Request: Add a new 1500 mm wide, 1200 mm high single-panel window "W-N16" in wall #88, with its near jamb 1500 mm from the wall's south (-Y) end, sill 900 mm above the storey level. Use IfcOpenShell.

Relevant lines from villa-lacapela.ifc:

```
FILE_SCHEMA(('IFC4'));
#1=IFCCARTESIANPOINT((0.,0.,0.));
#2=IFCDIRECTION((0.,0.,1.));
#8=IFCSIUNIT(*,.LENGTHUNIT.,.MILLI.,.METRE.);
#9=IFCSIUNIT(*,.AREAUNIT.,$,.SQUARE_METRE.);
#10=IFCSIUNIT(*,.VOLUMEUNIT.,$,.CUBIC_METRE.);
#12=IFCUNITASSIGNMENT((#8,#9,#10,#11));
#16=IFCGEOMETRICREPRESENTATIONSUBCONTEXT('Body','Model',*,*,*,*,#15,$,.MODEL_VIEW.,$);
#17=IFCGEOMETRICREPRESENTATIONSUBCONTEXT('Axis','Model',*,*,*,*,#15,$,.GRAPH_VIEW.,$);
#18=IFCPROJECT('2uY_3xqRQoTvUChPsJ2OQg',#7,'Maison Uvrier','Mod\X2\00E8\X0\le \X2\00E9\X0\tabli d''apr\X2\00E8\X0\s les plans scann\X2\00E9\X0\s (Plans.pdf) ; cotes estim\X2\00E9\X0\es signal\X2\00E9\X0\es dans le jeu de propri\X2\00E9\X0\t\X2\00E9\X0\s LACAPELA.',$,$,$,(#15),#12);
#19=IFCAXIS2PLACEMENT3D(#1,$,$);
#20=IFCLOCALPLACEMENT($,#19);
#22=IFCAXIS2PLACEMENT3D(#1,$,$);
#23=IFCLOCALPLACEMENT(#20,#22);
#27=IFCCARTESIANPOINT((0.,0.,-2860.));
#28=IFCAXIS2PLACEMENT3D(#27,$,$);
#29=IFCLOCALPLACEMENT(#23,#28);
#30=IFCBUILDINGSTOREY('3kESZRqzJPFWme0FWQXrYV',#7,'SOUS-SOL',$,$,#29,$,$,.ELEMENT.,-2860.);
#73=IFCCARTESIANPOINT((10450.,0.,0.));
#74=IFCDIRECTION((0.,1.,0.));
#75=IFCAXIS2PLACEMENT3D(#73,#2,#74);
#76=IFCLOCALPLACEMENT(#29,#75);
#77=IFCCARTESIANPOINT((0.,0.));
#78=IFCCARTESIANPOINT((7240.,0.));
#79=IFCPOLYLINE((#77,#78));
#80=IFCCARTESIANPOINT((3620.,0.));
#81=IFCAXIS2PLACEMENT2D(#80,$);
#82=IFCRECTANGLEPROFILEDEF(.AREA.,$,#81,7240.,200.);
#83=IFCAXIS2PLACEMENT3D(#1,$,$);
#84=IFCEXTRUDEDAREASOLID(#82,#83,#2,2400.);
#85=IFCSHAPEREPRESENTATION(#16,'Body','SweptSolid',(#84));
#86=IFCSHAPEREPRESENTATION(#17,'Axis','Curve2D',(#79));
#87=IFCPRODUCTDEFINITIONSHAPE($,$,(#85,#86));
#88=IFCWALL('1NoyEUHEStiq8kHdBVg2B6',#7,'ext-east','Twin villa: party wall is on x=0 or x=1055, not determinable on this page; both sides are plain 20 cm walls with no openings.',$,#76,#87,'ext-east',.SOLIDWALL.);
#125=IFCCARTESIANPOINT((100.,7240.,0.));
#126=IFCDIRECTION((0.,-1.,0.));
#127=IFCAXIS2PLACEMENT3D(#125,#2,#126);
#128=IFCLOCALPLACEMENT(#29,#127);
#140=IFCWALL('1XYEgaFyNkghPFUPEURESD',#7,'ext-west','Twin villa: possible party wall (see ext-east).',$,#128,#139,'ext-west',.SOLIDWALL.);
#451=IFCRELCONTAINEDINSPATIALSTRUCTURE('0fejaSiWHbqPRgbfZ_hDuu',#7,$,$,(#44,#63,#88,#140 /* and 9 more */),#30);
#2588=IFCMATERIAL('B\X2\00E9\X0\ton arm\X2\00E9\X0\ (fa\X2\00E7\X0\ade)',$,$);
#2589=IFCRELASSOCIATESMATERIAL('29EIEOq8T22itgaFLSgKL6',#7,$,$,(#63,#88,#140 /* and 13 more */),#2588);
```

```python
import numpy as np
import ifcopenshell
import ifcopenshell.api.feature
import ifcopenshell.api.geometry
import ifcopenshell.api.root
import ifcopenshell.api.spatial
import ifcopenshell.geom
import ifcopenshell.util.element
import ifcopenshell.util.placement
import ifcopenshell.util.representation
import ifcopenshell.util.shape
import ifcopenshell.util.unit

model = ifcopenshell.open("villa-lacapela.ifc")
unit_scale = ifcopenshell.util.unit.calculate_unit_scale(model)
settings = ifcopenshell.geom.settings()


def volume(element):
    """Net volume in cubic metres, openings subtracted."""
    shape = ifcopenshell.geom.create_shape(settings, element)
    return ifcopenshell.util.shape.get_volume(shape.geometry)


wall = model.by_guid("1NoyEUHEStiq8kHdBVg2B6")
storey = ifcopenshell.util.element.get_container(wall, ifc_class="IfcBuildingStorey")
context = ifcopenshell.util.representation.get_context(model, "Model", "Body", "MODEL_VIEW")
before = volume(wall)

width, height, from_end, sill = 1.5, 1.2, 1.5, 0.9  # metres

# The wall runs along its own X axis, and the end named is its -X end.
wall_shape = ifcopenshell.geom.create_shape(settings, wall)
x, y, z = ifcopenshell.util.shape.get_vertices(wall_shape.geometry).T
start = x.min() + from_end
face, thickness = float(y.min()), float(y.max() - y.min())
wall_matrix = ifcopenshell.util.placement.get_local_placement(wall.ObjectPlacement)
level = ifcopenshell.util.placement.get_local_placement(storey.ObjectPlacement)[2, 3]


def in_wall(x, y):
    """Placement at x, y metres in the wall's axes, at sill height."""
    matrix = wall_matrix.copy()
    matrix[:, 3] = wall_matrix @ np.array([x / unit_scale, y / unit_scale, 0.0, 1.0])
    matrix[2, 3] = level + sill / unit_scale
    return matrix


# Opening: a box that overshoots both wall faces by 50 mm.
opening = ifcopenshell.api.root.create_entity(model, ifc_class="IfcOpeningElement", predefined_type="OPENING")
box = ifcopenshell.api.geometry.add_wall_representation(
    model, context=context, length=width, height=height, thickness=thickness + 0.1
)
ifcopenshell.api.geometry.assign_representation(model, product=opening, representation=box)
ifcopenshell.api.geometry.edit_object_placement(model, product=opening, matrix=in_wall(start, face - 0.05), is_si=False)
ifcopenshell.api.feature.add_feature(model, feature=opening, element=wall)

window = ifcopenshell.api.root.create_entity(model, ifc_class="IfcWindow", name="W-N16", predefined_type="WINDOW")
window.OverallWidth, window.OverallHeight = width / unit_scale, height / unit_scale
window.PartitioningType = "SINGLE_PANEL"
body = ifcopenshell.api.geometry.add_window_representation(
    model,
    context=context,
    overall_width=window.OverallWidth,
    overall_height=window.OverallHeight,
    partition_type="SINGLE_PANEL",
)
ifcopenshell.api.geometry.assign_representation(model, product=window, representation=body)
ifcopenshell.api.spatial.assign_container(model, products=[window], relating_structure=storey)
ifcopenshell.api.feature.add_filling(model, opening=opening, element=window)

# Centre the window in the wall's thickness.
ifcopenshell.api.geometry.edit_object_placement(model, product=window, matrix=in_wall(start, face), is_si=False)
window_shape = ifcopenshell.geom.create_shape(settings, window)
depth = ifcopenshell.util.shape.get_vertices(window_shape.geometry)[:, 1]
offset = face + thickness / 2 - (depth.min() + depth.max()) / 2
ifcopenshell.api.geometry.edit_object_placement(model, product=window, matrix=in_wall(start, offset), is_si=False)

after = volume(wall)

print(f"wall volume {before:.3f} -> {after:.3f} m3")

model.write("villa-lacapela_rev.ifc")
```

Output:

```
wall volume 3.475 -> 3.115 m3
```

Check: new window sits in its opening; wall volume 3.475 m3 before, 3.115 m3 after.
